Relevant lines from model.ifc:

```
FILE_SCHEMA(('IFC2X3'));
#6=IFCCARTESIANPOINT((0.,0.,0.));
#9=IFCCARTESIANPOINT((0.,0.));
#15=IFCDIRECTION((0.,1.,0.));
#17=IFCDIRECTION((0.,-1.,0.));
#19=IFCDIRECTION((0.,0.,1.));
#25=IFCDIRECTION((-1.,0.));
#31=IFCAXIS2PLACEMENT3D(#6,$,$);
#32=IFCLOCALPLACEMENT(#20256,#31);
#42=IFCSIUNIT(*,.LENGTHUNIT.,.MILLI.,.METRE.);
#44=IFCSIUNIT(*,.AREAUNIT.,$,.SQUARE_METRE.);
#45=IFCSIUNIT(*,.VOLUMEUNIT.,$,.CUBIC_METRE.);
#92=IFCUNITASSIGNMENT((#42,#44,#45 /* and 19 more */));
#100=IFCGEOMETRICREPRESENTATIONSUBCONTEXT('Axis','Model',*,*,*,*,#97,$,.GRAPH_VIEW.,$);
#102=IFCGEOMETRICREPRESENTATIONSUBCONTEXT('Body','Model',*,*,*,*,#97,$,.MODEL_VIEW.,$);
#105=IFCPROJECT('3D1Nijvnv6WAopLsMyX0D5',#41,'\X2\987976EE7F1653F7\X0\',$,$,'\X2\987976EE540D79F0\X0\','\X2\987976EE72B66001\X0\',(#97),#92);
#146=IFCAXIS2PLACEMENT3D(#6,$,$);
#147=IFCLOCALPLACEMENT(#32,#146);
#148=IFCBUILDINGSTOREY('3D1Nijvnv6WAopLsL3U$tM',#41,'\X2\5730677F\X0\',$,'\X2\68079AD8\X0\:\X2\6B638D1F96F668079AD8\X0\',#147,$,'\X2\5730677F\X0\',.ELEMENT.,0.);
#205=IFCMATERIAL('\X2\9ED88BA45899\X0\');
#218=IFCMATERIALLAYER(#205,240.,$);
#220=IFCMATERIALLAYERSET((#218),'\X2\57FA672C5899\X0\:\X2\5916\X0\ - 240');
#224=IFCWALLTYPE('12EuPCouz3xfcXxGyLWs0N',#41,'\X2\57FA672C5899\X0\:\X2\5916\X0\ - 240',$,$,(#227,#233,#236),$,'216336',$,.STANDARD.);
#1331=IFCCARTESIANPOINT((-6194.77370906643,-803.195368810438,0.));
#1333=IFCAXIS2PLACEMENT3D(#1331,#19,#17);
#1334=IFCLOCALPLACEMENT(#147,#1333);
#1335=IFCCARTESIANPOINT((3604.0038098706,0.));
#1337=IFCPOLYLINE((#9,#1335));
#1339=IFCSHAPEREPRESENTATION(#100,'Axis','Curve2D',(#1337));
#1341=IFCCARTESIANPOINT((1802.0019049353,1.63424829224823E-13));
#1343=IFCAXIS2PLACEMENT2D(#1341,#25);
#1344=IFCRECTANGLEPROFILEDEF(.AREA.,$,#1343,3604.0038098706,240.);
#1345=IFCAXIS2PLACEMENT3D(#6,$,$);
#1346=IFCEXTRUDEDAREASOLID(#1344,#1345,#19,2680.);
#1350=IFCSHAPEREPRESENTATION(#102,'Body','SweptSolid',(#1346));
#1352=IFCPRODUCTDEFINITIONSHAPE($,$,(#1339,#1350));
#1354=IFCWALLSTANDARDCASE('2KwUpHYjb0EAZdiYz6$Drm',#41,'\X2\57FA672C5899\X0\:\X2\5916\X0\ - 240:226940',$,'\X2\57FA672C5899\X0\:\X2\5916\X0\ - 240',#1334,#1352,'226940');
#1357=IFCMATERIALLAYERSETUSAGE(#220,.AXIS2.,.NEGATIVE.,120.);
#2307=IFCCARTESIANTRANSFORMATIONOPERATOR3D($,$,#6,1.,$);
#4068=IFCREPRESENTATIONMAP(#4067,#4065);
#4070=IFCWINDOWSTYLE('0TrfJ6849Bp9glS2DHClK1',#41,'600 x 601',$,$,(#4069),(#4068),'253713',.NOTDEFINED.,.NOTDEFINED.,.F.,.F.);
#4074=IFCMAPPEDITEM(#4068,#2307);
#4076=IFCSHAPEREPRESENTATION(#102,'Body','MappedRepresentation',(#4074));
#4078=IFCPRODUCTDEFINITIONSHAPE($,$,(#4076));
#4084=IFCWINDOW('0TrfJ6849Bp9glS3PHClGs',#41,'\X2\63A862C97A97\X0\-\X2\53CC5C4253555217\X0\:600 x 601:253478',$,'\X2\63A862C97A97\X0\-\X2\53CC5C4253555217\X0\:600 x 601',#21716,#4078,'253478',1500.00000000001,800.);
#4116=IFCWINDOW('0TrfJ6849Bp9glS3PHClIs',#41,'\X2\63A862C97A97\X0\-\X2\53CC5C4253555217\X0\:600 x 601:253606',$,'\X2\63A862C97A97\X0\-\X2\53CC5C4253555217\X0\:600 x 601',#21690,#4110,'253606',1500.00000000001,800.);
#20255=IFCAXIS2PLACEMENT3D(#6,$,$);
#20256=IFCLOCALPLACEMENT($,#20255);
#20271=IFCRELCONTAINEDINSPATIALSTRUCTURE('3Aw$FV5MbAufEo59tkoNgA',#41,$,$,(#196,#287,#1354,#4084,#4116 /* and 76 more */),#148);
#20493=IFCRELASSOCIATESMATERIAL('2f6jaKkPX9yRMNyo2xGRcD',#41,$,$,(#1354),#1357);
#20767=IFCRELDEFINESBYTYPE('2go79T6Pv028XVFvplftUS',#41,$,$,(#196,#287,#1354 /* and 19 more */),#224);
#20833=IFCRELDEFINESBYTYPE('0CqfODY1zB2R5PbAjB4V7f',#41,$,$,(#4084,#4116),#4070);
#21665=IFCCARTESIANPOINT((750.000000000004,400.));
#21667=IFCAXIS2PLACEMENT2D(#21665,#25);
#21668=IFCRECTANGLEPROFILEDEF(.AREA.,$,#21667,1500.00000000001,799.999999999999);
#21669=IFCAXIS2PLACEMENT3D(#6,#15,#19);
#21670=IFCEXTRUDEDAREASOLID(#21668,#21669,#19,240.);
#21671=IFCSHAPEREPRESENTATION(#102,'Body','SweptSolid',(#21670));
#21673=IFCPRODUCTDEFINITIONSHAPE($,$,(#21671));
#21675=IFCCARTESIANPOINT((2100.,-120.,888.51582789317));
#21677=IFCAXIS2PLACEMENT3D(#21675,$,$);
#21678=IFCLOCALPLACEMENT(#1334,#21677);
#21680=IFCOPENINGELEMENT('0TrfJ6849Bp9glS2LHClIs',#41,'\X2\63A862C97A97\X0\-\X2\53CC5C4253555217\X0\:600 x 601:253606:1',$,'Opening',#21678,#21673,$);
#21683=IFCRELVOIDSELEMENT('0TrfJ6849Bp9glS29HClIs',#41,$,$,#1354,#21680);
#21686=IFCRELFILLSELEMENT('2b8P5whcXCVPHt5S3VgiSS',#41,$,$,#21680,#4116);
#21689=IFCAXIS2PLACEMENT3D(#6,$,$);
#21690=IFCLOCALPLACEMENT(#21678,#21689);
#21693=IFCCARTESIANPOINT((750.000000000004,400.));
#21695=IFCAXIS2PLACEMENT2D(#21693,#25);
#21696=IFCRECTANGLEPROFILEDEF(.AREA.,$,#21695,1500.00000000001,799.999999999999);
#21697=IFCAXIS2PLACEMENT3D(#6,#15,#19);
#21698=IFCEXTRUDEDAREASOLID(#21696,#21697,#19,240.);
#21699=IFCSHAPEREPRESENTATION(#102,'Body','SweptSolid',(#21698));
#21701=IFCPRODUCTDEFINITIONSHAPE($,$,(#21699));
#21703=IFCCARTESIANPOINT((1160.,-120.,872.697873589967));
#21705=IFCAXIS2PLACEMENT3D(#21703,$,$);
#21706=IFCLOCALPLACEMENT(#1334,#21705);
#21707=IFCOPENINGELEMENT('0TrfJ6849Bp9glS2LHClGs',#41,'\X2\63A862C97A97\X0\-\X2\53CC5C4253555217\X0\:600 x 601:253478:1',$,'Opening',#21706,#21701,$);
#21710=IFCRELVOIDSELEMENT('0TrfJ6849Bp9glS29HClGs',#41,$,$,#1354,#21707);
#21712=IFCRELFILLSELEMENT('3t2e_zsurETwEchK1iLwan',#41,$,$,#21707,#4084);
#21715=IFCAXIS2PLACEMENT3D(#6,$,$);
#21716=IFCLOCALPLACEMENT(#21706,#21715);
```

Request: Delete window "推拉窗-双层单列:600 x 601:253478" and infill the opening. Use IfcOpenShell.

```python
import ifcopenshell
import ifcopenshell.api.feature
import ifcopenshell.api.root
import ifcopenshell.geom
import ifcopenshell.util.shape

model = ifcopenshell.open("model.ifc")
settings = ifcopenshell.geom.settings()


def volume(element):
    """Net volume in cubic metres, openings subtracted."""
    shape = ifcopenshell.geom.create_shape(settings, element)
    return ifcopenshell.util.shape.get_volume(shape.geometry)


window = model.by_id(4084)
opening = window.FillsVoids[0].RelatingOpeningElement
wall = opening.VoidsElements[0].RelatingBuildingElement
before = volume(wall)

ifcopenshell.api.root.remove_product(model, product=window)
ifcopenshell.api.feature.remove_feature(model, feature=opening)

after = volume(wall)

print(f"wall volume {before:.3f} -> {after:.3f} m3")

model.write("model_edited.ifc")
```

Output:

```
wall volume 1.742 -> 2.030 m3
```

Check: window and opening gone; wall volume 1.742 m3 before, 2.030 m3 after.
